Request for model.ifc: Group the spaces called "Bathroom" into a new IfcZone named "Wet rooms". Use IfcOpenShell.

First a look at what the model holds.

```python
import ifcopenshell

model = ifcopenshell.open("model.ifc")
print(model.schema)
seen = {}
for space in model.by_type("IfcSpace"):
    seen[space.LongName] = seen.get(space.LongName, 0) + 1
for name, count in sorted(seen.items(), key=str):
    print(count, "x", name)
print("zones:", [z.Name for z in model.by_type("IfcZone")][:20])
```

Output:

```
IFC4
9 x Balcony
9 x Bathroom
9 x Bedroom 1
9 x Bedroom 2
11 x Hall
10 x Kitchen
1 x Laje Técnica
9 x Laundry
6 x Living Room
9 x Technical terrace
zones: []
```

```python
import ifcopenshell
import ifcopenshell.api.group
import ifcopenshell.api.root

model = ifcopenshell.open("model.ifc")

names = {"Bathroom"}
spaces = [s for s in model.by_type("IfcSpace") if s.LongName in names]

zone = ifcopenshell.api.root.create_entity(model, ifc_class="IfcZone", name="Wet rooms")
ifcopenshell.api.group.assign_group(model, products=spaces, group=zone)
print(len(spaces), "spaces in", zone.Name)

model.write("model_updated.ifc")
```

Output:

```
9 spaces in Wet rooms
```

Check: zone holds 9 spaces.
